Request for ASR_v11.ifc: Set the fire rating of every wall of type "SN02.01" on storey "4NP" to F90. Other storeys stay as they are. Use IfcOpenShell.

First a look at what the model holds.

```python
import ifcopenshell
import ifcopenshell.util.element

model = ifcopenshell.open("ASR_v11.ifc")
print(model.schema)
storey = next(s for s in model.by_type("IfcBuildingStorey") if s.Name == "4NP")
walls = [e for e in ifcopenshell.util.element.get_decomposition(storey) if e.is_a("IfcWall")]
seen = {}
for e in walls:
    element_type = ifcopenshell.util.element.get_type(e)
    key = (element_type.Name if element_type != e and element_type else None, ifcopenshell.util.element.get_pset(e, "Pset_WallCommon", "FireRating"))
    seen[key] = seen.get(key, 0) + 1
for (name, value), count in sorted(seen.items(), key=str):
    print(count, "x", name, "|", value)
```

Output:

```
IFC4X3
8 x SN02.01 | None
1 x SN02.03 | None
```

```python
import ifcopenshell
import ifcopenshell.api.pset
import ifcopenshell.util.element

model = ifcopenshell.open("ASR_v11.ifc")

storey = next(s for s in model.by_type("IfcBuildingStorey") if s.Name == "4NP")
walls = [e for e in ifcopenshell.util.element.get_decomposition(storey) if e.is_a("IfcWall")]

count = 0
for e in walls:
    element_type = ifcopenshell.util.element.get_type(e)
    if element_type in (None, e) or element_type.Name != "SN02.01":
        continue
    # add_pset returns the element's existing set when there is one.
    pset = ifcopenshell.api.pset.add_pset(model, product=e, name="Pset_WallCommon")
    ifcopenshell.api.pset.edit_pset(model, pset=pset, properties={"FireRating": "F90"})
    count += 1

print(count, "walls updated")

model.write("ASR_v11_edited.ifc")
```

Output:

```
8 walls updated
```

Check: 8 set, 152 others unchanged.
